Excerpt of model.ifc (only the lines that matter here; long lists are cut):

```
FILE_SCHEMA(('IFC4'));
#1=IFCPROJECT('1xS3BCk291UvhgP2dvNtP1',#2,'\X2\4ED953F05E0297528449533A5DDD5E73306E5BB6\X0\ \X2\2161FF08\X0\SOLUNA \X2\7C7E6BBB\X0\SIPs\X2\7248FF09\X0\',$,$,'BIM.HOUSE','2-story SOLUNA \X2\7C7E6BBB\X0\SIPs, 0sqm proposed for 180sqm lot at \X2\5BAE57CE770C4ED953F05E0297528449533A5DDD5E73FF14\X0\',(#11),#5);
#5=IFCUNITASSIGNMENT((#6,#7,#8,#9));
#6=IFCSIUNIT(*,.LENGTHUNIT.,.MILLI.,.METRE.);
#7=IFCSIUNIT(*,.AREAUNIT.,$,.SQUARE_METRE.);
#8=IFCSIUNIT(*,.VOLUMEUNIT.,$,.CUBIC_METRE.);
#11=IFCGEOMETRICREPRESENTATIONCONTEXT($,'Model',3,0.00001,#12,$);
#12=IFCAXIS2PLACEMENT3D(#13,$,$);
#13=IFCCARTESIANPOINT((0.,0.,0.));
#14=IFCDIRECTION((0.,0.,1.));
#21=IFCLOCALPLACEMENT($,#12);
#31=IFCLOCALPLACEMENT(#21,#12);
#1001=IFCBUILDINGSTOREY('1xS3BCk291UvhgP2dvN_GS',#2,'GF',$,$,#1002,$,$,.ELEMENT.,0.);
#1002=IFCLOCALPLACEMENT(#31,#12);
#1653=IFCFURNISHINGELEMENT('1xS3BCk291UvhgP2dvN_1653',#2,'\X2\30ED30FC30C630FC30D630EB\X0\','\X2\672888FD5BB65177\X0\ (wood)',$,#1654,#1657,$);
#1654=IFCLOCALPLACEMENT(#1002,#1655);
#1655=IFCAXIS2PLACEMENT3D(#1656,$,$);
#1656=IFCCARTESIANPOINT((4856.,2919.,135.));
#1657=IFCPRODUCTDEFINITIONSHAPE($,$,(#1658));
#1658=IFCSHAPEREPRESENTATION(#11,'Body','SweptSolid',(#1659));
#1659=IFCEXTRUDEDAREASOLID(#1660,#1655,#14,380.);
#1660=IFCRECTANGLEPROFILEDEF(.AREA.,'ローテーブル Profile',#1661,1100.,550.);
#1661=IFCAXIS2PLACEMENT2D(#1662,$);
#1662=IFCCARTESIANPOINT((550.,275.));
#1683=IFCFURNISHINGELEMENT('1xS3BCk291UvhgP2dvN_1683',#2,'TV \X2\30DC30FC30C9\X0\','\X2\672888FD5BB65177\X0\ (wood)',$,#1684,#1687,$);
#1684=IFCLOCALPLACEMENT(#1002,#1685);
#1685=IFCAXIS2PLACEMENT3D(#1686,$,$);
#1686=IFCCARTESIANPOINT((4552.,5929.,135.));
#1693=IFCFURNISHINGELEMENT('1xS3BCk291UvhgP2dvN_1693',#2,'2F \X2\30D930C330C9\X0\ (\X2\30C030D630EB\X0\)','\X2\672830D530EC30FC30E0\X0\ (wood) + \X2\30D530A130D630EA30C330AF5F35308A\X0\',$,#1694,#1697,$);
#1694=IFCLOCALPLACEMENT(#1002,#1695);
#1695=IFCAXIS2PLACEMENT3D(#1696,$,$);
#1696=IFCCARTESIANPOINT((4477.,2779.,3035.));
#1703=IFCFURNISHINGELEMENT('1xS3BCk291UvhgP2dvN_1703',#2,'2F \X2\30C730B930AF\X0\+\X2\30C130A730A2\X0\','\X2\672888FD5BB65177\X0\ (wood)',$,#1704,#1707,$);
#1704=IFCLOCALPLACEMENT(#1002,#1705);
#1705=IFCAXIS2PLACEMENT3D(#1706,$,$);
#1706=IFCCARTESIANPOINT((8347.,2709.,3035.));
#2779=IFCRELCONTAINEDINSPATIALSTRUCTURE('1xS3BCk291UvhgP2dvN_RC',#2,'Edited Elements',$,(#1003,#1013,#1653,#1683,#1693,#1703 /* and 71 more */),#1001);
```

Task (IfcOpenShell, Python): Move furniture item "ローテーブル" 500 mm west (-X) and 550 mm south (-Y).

```python
import ifcopenshell
import ifcopenshell.api.geometry
import ifcopenshell.util.placement

model = ifcopenshell.open("model.ifc")

item = model.by_id(1653)
matrix = ifcopenshell.util.placement.get_local_placement(item.ObjectPlacement)
matrix[0, 3] -= 500.0
matrix[1, 3] -= 550.0
ifcopenshell.api.geometry.edit_object_placement(model, product=item, matrix=matrix, is_si=False)

print(ifcopenshell.util.placement.get_local_placement(item.ObjectPlacement).round(3) + 0.0)

model.write("model-out.ifc")
```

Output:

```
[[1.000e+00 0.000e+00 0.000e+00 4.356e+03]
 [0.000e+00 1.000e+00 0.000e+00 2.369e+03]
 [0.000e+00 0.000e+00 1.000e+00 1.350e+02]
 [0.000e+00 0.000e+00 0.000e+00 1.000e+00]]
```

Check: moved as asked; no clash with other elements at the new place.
